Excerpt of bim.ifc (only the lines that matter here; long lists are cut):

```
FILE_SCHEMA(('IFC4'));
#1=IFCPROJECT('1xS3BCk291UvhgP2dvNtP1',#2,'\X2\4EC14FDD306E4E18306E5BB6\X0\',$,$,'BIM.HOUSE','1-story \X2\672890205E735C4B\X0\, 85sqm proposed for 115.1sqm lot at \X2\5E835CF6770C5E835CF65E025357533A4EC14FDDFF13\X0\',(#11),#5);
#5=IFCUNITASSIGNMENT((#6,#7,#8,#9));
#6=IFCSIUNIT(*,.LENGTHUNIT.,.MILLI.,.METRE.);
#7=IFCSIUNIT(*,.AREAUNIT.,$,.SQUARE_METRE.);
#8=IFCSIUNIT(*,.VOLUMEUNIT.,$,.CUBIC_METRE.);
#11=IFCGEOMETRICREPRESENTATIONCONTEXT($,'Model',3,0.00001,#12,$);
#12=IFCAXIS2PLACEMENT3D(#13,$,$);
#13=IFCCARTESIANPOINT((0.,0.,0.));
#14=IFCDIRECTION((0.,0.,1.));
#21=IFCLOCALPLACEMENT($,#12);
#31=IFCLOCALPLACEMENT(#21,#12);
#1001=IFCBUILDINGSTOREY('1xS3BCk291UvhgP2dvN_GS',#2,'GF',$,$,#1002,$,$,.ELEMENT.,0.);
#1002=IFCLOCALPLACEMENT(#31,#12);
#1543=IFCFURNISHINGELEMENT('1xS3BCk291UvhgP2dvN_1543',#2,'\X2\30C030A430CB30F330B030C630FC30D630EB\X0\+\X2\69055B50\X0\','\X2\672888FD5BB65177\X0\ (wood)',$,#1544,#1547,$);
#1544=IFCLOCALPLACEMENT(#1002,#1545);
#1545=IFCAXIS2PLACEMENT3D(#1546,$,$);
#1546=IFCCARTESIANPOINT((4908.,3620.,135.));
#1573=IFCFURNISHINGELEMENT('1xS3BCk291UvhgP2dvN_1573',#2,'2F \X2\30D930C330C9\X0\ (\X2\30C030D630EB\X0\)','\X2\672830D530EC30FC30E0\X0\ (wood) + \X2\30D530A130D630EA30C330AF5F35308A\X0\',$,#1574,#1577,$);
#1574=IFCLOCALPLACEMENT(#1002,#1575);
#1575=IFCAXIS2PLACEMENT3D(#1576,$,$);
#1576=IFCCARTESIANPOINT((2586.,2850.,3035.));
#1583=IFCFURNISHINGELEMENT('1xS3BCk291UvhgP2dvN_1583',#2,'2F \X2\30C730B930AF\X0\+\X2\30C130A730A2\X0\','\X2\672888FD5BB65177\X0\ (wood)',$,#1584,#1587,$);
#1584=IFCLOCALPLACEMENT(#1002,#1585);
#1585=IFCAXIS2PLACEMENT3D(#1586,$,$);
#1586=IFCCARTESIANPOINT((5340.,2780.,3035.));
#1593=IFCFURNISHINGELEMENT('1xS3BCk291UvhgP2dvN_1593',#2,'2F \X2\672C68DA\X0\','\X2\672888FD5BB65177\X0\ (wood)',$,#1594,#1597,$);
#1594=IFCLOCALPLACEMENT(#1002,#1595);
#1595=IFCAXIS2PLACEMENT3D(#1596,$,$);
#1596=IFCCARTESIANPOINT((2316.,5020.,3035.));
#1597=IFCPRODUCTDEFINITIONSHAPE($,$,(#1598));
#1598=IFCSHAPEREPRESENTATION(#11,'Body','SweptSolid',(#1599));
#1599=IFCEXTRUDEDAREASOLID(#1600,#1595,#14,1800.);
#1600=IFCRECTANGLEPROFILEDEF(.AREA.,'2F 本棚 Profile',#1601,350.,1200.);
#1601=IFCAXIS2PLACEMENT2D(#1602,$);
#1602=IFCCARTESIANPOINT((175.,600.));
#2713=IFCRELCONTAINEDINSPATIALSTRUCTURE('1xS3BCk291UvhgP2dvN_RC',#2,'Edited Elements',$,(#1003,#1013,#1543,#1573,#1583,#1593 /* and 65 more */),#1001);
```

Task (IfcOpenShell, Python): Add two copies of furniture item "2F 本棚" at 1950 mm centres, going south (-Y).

```python
import numpy as np
import ifcopenshell
import ifcopenshell.api.geometry
import ifcopenshell.api.root
import ifcopenshell.util.element
import ifcopenshell.util.placement
import ifcopenshell.util.unit

model = ifcopenshell.open("bim.ifc")
unit_scale = ifcopenshell.util.unit.calculate_unit_scale(model)


def reuse_history(source, copy):
    """copy_class also copies each property set's owner history, people and application; keep the originals."""
    for rel in copy.IsDefinedBy:
        if rel.is_a("IfcRelDefinesByProperties") and (history := rel.RelatingPropertyDefinition.OwnerHistory):
            rel.RelatingPropertyDefinition.OwnerHistory = source.OwnerHistory
            ifcopenshell.util.element.remove_deep2(model, history)


source = model.by_guid("1xS3BCk291UvhgP2dvN_1593")
base = ifcopenshell.util.placement.get_local_placement(source.ObjectPlacement)
step = np.array([0.0, -1.0, 0.0]) * 1.95 / unit_scale

for i in range(1, 3):
    copy = ifcopenshell.api.root.copy_class(model, product=source)
    copy.Representation = ifcopenshell.util.element.copy_deep(
        model, source.Representation, exclude=["IfcGeometricRepresentationContext", "IfcRepresentationMap"]
    )
    reuse_history(source, copy)
    matrix = base.copy()
    matrix[:3, 3] += i * step
    print("added at", matrix[:3, 3].round(3) + 0.0)
    ifcopenshell.api.geometry.edit_object_placement(model, product=copy, matrix=matrix, is_si=False)

model.write("bim_v2.ifc")
```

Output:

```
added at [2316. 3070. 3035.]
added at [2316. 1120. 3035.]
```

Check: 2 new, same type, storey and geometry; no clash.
